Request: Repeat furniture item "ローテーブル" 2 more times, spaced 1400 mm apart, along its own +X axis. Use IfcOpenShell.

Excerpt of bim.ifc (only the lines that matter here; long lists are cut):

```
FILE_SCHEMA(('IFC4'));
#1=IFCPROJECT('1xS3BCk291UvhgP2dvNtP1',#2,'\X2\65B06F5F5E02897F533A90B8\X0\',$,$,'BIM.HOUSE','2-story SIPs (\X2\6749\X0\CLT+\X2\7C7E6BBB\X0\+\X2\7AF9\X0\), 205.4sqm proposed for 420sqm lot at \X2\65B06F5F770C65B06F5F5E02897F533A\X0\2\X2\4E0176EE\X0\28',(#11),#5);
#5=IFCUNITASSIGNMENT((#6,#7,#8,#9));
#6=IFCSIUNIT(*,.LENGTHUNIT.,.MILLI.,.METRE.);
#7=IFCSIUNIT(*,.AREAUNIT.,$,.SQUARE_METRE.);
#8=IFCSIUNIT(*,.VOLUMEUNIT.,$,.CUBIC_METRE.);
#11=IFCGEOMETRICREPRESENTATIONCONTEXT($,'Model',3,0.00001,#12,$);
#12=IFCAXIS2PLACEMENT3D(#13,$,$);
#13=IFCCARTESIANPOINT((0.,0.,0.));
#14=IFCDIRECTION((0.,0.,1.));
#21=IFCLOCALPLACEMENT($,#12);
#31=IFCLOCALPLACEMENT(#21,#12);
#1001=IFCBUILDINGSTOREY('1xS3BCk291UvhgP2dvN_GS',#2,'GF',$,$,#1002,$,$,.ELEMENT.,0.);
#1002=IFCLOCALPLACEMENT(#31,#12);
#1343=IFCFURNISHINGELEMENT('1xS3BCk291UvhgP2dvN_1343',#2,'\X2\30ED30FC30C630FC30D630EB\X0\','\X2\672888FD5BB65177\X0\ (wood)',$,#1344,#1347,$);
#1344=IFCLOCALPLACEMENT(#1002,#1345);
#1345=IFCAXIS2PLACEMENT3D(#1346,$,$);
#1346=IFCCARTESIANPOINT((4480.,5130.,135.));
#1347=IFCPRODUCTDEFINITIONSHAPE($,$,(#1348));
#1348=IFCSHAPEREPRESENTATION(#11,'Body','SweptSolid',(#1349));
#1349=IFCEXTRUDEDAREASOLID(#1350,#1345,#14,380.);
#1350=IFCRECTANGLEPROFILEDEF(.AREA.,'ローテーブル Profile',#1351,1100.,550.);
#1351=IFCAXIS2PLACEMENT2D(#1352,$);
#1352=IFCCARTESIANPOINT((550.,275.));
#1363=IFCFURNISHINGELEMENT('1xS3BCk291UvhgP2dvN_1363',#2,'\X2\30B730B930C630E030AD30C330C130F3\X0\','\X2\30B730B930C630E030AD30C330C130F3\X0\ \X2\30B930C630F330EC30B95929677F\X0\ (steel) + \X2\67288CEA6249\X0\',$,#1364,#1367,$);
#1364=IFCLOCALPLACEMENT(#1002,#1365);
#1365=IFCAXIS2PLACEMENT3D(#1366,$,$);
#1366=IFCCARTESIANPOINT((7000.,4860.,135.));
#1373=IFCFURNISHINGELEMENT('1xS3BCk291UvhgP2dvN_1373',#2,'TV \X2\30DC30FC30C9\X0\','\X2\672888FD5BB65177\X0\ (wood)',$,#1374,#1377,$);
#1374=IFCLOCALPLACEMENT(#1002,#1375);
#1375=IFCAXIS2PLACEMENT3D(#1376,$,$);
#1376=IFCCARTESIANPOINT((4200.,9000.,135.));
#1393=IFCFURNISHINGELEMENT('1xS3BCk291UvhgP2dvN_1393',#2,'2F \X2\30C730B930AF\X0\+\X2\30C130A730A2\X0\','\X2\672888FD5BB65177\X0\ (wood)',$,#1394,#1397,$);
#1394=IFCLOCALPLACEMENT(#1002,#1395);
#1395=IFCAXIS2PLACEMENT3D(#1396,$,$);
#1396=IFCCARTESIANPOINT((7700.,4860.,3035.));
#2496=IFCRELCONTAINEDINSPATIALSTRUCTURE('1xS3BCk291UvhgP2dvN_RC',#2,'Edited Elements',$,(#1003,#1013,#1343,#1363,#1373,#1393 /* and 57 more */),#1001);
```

```python
import ifcopenshell
import ifcopenshell.api.geometry
import ifcopenshell.api.root
import ifcopenshell.util.element
import ifcopenshell.util.placement
import ifcopenshell.util.unit

model = ifcopenshell.open("bim.ifc")
unit_scale = ifcopenshell.util.unit.calculate_unit_scale(model)


def reuse_history(source, copy):
    """copy_class also copies each property set's owner history, people and application; keep the originals."""
    for rel in copy.IsDefinedBy:
        if rel.is_a("IfcRelDefinesByProperties") and (history := rel.RelatingPropertyDefinition.OwnerHistory):
            rel.RelatingPropertyDefinition.OwnerHistory = source.OwnerHistory
            ifcopenshell.util.element.remove_deep2(model, history)


source = model.by_guid("1xS3BCk291UvhgP2dvN_1343")
base = ifcopenshell.util.placement.get_local_placement(source.ObjectPlacement)
step = base[:3, 0] * 1.4 / unit_scale

for i in range(1, 3):
    copy = ifcopenshell.api.root.copy_class(model, product=source)
    copy.Representation = ifcopenshell.util.element.copy_deep(
        model, source.Representation, exclude=["IfcGeometricRepresentationContext", "IfcRepresentationMap"]
    )
    reuse_history(source, copy)
    matrix = base.copy()
    matrix[:3, 3] += i * step
    print("added at", matrix[:3, 3].round(3) + 0.0)
    ifcopenshell.api.geometry.edit_object_placement(model, product=copy, matrix=matrix, is_si=False)

model.write("bim_rev.ifc")
```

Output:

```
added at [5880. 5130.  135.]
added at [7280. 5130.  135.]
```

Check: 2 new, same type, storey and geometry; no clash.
